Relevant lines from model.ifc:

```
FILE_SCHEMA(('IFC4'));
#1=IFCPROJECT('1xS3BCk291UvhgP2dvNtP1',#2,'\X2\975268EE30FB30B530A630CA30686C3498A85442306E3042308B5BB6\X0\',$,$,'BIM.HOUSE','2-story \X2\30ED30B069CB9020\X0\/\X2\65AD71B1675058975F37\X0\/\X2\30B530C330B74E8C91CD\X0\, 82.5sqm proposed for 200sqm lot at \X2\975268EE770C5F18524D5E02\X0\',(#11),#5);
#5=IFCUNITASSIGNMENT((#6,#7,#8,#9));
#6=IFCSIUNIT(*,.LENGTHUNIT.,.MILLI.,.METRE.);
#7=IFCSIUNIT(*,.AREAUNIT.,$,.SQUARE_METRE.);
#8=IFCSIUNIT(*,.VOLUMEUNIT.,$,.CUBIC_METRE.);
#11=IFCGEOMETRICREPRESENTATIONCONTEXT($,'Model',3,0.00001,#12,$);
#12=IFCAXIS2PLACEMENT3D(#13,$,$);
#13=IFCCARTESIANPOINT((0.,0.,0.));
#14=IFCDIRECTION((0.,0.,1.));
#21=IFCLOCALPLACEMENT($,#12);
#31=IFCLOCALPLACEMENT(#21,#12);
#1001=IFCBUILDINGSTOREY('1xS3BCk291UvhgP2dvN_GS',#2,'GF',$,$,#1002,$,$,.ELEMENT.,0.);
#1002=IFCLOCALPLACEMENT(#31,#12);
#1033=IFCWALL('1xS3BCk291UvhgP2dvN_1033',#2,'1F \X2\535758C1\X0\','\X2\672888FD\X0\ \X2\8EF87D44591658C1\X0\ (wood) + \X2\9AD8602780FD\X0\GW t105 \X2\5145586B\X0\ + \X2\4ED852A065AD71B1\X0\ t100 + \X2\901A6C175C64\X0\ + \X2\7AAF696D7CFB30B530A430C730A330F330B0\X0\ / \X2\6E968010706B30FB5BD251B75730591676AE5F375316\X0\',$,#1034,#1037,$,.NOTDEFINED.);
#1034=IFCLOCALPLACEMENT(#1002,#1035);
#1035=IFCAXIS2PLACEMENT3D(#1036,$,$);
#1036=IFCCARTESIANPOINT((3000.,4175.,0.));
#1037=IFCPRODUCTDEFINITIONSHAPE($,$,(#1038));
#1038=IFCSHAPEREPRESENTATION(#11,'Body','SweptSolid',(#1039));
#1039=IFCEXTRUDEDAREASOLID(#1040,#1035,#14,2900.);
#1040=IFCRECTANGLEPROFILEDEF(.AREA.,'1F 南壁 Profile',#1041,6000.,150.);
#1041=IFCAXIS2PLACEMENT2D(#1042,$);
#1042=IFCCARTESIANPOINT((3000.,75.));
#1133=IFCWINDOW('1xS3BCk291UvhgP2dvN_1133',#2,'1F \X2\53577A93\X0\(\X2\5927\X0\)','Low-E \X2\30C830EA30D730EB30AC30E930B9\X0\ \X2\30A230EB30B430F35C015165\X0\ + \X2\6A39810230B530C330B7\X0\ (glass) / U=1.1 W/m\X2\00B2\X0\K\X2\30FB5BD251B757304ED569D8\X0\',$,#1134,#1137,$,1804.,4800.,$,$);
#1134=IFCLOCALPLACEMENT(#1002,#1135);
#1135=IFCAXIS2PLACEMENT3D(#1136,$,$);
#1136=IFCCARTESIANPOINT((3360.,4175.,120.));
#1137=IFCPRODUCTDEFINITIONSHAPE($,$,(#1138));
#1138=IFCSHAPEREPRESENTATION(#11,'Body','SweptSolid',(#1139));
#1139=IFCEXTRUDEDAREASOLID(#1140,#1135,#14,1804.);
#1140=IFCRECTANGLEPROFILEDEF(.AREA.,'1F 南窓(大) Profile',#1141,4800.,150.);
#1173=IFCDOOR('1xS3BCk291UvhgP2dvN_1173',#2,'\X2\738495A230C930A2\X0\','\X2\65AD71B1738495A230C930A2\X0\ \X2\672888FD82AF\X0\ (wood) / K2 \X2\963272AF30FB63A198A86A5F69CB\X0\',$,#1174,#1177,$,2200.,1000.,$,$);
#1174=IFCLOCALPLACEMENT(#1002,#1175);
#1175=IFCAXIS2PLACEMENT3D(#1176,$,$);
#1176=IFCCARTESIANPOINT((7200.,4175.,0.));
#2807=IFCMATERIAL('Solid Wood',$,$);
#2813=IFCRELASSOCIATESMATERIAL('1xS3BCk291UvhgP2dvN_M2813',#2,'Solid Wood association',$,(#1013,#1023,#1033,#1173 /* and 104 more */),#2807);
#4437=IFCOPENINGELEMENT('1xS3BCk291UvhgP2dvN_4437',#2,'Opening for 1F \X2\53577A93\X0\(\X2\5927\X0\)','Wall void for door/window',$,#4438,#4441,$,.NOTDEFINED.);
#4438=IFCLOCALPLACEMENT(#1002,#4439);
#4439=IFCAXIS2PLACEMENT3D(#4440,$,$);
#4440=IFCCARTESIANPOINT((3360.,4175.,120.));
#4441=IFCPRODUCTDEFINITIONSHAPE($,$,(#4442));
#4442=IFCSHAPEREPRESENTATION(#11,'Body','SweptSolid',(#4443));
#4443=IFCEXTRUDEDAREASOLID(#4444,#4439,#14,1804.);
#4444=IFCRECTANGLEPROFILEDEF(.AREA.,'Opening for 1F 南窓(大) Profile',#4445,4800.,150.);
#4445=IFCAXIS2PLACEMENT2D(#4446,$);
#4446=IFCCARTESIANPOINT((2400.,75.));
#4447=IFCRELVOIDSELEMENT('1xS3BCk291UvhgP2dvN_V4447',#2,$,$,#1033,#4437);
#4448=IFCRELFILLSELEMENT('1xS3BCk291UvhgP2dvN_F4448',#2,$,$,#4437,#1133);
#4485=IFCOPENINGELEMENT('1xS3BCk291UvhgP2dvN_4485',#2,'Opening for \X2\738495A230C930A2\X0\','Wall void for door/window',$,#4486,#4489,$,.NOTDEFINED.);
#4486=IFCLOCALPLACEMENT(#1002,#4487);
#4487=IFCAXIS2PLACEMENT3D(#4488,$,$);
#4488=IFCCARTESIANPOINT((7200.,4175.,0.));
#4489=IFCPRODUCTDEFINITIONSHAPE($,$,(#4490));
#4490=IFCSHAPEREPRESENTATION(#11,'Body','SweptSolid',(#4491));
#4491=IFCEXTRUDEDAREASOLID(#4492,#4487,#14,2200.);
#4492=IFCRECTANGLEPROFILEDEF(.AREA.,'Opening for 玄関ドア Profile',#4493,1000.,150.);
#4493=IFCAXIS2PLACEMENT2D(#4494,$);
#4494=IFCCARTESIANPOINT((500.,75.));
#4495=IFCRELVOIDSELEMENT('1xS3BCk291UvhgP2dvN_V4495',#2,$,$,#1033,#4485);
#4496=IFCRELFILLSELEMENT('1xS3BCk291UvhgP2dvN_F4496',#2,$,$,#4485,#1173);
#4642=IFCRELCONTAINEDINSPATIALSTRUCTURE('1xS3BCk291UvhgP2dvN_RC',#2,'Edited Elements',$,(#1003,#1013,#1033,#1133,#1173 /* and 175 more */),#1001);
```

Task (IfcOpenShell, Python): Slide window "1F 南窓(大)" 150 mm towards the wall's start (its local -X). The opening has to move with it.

```python
import ifcopenshell
import ifcopenshell.api.geometry
import ifcopenshell.util.placement
import ifcopenshell.util.unit

model = ifcopenshell.open("model.ifc")
unit_scale = ifcopenshell.util.unit.calculate_unit_scale(model)

window = model.by_guid("1xS3BCk291UvhgP2dvN_1133")
opening = window.FillsVoids[0].RelatingOpeningElement
wall = opening.VoidsElements[0].RelatingBuildingElement

wall_matrix = ifcopenshell.util.placement.get_local_placement(wall.ObjectPlacement)
shift = wall_matrix[:3, 0] * -0.15 / unit_scale
before = ifcopenshell.util.placement.get_local_placement(window.ObjectPlacement)[:3, 3].copy()

# The window is not placed relative to its opening, so move both.
for product in (opening, window):
    matrix = ifcopenshell.util.placement.get_local_placement(product.ObjectPlacement)
    matrix[:3, 3] += shift
    ifcopenshell.api.geometry.edit_object_placement(model, product=product, matrix=matrix, is_si=False)

after = ifcopenshell.util.placement.get_local_placement(window.ObjectPlacement)[:3, 3]
print("window moved by", (after - before).round(3) + 0.0)

model.write("model-out.ifc")
```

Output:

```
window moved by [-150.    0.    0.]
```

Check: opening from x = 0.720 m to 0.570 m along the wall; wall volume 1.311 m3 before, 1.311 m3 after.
